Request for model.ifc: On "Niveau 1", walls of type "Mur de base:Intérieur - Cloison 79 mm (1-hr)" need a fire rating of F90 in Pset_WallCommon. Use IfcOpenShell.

First a look at what the model holds.

```python
import ifcopenshell
import ifcopenshell.util.element

model = ifcopenshell.open("model.ifc")
print(model.schema)
storey = next(s for s in model.by_type("IfcBuildingStorey") if s.Name == "Niveau 1")
walls = [e for e in ifcopenshell.util.element.get_decomposition(storey) if e.is_a("IfcWall")]
seen = {}
for e in walls:
    element_type = ifcopenshell.util.element.get_type(e)
    key = (element_type.Name if element_type != e and element_type else None, ifcopenshell.util.element.get_pset(e, "Pset_WallCommon", "FireRating"))
    seen[key] = seen.get(key, 0) + 1
for (name, value), count in sorted(seen.items(), key=str):
    print(count, "x", name, "|", value)
```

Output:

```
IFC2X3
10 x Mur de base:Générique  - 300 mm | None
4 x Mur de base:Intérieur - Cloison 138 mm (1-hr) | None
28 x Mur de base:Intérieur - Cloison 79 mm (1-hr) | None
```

```python
import ifcopenshell
import ifcopenshell.api.pset
import ifcopenshell.util.element

model = ifcopenshell.open("model.ifc")

storey = next(s for s in model.by_type("IfcBuildingStorey") if s.Name == "Niveau 1")
walls = [e for e in ifcopenshell.util.element.get_decomposition(storey) if e.is_a("IfcWall")]

count = 0
for e in walls:
    element_type = ifcopenshell.util.element.get_type(e)
    if element_type in (None, e) or element_type.Name != 'Mur de base:Intérieur - Cloison 79\xa0mm (1-hr)':
        continue
    # add_pset returns the element's existing set when there is one.
    pset = ifcopenshell.api.pset.add_pset(model, product=e, name="Pset_WallCommon")
    ifcopenshell.api.pset.edit_pset(model, pset=pset, properties={"FireRating": "F90"})
    count += 1

print(count, "walls updated")

model.write("model_updated.ifc")
```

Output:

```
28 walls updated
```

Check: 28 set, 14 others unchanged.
